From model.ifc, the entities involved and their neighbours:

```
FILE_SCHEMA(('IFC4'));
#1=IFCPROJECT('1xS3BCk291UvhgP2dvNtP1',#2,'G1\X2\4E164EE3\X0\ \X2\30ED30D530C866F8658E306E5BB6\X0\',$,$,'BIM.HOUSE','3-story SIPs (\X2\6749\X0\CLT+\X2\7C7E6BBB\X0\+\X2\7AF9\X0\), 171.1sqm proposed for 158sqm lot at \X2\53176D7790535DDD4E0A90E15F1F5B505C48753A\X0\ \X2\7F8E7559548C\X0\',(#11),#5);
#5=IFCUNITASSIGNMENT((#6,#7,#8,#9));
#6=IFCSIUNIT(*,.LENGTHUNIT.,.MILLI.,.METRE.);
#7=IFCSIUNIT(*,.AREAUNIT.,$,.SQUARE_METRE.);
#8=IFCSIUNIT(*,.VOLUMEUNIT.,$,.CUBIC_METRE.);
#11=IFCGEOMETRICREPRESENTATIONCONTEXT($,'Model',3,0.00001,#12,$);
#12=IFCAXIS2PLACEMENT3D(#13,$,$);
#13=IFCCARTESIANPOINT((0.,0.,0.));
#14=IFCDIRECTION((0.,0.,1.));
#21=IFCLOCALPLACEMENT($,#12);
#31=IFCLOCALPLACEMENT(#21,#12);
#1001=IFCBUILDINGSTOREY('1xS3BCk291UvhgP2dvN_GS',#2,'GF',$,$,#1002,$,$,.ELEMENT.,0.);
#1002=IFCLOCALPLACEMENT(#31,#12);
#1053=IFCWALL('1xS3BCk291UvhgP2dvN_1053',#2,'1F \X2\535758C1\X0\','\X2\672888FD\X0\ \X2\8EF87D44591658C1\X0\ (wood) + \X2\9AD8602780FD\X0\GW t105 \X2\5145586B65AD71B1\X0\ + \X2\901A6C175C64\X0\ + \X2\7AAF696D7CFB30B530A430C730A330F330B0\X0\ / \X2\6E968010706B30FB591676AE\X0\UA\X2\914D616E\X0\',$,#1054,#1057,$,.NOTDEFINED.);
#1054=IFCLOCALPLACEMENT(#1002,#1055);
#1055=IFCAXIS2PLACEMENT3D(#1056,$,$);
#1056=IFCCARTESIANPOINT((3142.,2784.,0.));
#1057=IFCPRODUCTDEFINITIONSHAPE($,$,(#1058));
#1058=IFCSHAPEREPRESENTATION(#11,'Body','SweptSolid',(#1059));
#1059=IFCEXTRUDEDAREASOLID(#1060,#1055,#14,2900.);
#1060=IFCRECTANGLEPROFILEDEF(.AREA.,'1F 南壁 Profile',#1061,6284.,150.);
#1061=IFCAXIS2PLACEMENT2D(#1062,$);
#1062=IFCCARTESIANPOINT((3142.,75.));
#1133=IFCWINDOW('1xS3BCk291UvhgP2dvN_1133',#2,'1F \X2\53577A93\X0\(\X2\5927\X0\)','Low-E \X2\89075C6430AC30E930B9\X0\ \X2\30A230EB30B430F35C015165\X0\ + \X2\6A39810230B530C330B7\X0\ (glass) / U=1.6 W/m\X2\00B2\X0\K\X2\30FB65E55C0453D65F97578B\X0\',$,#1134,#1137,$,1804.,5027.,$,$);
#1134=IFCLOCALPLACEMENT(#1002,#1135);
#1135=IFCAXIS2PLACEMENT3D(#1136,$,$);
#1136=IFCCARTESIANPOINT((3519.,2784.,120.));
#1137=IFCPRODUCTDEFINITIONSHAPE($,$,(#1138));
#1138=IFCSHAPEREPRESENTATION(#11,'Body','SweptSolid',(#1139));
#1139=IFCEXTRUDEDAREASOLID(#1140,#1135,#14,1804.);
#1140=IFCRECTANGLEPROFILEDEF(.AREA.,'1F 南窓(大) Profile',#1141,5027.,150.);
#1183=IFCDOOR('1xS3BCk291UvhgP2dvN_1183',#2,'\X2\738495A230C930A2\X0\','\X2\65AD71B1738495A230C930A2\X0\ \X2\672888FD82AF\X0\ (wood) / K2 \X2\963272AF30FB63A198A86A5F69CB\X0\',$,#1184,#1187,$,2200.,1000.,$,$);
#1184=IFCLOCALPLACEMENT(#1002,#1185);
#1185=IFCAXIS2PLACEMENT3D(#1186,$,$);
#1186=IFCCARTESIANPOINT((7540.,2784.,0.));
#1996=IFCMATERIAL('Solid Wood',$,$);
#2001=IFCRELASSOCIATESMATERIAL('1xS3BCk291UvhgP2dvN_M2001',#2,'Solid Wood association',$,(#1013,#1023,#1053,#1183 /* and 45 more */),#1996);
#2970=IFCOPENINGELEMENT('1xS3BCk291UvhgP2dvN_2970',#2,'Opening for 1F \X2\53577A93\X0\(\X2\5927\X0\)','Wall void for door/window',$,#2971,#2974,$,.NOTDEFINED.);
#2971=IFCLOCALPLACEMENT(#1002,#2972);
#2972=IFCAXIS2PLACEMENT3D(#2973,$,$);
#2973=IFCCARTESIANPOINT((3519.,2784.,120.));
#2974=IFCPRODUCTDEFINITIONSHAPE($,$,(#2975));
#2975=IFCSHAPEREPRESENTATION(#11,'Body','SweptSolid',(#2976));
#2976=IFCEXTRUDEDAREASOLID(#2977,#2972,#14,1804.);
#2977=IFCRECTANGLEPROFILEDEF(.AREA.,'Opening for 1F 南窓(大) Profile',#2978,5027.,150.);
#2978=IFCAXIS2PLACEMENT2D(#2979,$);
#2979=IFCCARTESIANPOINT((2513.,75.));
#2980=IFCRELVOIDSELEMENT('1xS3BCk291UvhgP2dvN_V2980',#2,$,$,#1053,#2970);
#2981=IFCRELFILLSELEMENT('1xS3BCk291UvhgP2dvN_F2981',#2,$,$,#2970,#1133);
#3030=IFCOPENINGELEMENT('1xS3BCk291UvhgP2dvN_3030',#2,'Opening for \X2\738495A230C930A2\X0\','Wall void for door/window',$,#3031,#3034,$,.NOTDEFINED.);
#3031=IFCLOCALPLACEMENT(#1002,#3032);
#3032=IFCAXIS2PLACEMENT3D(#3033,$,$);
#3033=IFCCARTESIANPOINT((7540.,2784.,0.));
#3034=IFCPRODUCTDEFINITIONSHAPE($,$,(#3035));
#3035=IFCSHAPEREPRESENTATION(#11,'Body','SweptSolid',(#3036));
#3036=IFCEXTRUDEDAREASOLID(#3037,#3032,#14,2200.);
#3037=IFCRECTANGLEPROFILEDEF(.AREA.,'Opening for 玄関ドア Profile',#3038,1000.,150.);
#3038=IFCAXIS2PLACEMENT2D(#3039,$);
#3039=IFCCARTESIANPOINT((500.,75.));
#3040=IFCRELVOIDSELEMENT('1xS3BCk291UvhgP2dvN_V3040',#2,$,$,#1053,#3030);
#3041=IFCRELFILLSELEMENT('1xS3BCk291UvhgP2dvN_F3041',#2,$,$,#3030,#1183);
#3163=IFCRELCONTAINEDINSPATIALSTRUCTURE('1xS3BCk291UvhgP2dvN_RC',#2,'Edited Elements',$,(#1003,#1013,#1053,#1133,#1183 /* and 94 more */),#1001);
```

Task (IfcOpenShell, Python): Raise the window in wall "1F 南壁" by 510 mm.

```python
import numpy as np
import ifcopenshell
import ifcopenshell.api.geometry
import ifcopenshell.util.placement
import ifcopenshell.util.unit

model = ifcopenshell.open("model.ifc")
unit_scale = ifcopenshell.util.unit.calculate_unit_scale(model)

window = model.by_id(1133)
opening = window.FillsVoids[0].RelatingOpeningElement
dz = 510.0

shift = np.array([0.0, 0.0, dz])
# The window is not placed relative to its opening, so move both.
for product in (opening, window):
    matrix = ifcopenshell.util.placement.get_local_placement(product.ObjectPlacement)
    matrix[:3, 3] += shift
    ifcopenshell.api.geometry.edit_object_placement(model, product=product, matrix=matrix, is_si=False)

print(f"moved by {dz * unit_scale:+.3f} m")

model.write("model_edited.ifc")
```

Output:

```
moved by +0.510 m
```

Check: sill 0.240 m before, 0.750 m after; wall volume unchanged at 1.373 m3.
